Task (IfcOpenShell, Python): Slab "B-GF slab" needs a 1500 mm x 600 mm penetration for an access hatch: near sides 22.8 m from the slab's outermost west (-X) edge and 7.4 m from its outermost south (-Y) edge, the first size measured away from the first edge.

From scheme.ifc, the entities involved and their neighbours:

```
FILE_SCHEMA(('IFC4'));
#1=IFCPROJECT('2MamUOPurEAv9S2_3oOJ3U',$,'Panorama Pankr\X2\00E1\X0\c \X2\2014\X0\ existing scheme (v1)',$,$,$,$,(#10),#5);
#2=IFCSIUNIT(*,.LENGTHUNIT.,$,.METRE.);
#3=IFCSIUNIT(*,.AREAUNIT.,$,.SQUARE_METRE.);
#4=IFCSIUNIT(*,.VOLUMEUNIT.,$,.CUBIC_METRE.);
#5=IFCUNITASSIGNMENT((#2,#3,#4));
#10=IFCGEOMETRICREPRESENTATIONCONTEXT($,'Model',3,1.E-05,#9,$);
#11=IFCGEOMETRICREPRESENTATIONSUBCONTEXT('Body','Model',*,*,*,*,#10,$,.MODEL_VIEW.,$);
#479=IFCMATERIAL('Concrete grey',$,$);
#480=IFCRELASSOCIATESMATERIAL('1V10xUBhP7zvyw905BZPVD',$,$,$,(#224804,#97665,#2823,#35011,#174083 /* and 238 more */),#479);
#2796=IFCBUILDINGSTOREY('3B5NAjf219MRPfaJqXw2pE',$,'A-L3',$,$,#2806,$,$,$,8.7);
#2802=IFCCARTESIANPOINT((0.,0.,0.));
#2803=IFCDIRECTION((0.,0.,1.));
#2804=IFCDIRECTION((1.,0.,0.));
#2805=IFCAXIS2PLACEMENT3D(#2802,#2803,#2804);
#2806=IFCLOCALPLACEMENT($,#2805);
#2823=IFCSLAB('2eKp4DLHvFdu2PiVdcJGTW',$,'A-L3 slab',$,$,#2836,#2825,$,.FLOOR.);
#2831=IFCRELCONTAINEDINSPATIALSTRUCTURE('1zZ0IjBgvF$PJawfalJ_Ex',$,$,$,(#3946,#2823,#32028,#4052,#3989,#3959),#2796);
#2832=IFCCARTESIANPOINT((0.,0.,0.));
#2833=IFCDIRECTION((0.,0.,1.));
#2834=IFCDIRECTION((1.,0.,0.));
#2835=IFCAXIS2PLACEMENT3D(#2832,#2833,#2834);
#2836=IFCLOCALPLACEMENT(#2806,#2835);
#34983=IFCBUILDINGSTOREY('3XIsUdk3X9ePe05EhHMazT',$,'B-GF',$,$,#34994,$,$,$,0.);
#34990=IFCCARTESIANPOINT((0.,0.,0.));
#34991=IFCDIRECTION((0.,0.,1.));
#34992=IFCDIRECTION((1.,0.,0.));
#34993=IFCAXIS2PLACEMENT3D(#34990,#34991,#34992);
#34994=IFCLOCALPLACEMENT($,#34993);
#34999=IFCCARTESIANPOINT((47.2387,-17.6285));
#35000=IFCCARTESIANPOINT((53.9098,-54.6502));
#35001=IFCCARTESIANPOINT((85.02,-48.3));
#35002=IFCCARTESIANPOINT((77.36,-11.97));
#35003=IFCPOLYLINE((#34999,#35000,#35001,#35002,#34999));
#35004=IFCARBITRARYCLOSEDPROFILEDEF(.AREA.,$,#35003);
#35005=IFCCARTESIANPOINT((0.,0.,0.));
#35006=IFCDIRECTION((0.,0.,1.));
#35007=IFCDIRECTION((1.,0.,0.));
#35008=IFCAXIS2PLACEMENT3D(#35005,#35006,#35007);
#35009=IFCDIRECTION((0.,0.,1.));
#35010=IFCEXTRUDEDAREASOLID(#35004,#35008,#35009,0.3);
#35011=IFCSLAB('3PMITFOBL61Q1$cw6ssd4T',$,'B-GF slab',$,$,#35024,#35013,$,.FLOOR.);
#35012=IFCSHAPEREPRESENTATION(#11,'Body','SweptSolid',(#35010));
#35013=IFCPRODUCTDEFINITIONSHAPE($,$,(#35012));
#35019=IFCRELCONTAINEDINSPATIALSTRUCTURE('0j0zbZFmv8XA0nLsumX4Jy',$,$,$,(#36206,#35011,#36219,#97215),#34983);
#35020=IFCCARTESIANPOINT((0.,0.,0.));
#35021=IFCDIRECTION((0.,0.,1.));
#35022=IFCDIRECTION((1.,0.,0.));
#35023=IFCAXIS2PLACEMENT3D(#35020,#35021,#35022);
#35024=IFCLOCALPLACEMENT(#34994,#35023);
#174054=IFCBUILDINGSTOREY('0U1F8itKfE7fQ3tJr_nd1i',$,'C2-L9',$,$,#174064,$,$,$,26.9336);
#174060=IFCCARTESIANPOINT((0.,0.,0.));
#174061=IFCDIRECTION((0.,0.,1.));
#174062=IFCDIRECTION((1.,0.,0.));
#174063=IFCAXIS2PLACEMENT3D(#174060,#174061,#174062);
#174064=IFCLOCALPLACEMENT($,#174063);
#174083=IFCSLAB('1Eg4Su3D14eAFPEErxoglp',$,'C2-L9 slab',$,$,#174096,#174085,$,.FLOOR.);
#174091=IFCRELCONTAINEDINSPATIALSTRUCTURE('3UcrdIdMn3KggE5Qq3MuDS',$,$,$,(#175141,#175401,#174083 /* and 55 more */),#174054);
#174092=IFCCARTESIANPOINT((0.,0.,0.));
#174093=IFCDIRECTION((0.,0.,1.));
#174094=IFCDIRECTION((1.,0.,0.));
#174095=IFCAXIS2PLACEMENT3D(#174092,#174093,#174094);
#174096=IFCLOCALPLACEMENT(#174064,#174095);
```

```python
import numpy as np
import ifcopenshell
import ifcopenshell.api.feature
import ifcopenshell.api.geometry
import ifcopenshell.api.root
import ifcopenshell.geom
import ifcopenshell.util.placement
import ifcopenshell.util.representation
import ifcopenshell.util.shape
import ifcopenshell.util.unit

model = ifcopenshell.open("scheme.ifc")
unit_scale = ifcopenshell.util.unit.calculate_unit_scale(model)
settings = ifcopenshell.geom.settings()


def volume(element):
    """Net volume in cubic metres, openings subtracted."""
    shape = ifcopenshell.geom.create_shape(settings, element)
    return ifcopenshell.util.shape.get_volume(shape.geometry)


slab = model.by_guid("3PMITFOBL61Q1$cw6ssd4T")
before = volume(slab)

# Extent in the slab's own axes, in metres. The edges named are its -X and -Y sides.
slab_shape = ifcopenshell.geom.create_shape(settings, slab)
vertices = ifcopenshell.util.shape.get_vertices(slab_shape.geometry)
x_min, y_min, bottom = vertices.min(axis=0)
top = vertices[:, 2].max()

opening = ifcopenshell.api.root.create_entity(model, ifc_class="IfcOpeningElement", name="Access hatch opening", predefined_type="OPENING")
context = ifcopenshell.util.representation.get_context(model, "Model", "Body", "MODEL_VIEW")
width, depth = 1.5, 0.6
outline = [(0.0, 0.0), (width, 0.0), (width, depth), (0.0, depth), (0.0, 0.0)]
# Overshoot both faces by 50 mm so the cut is clean.
shape = ifcopenshell.api.geometry.add_slab_representation(
    model, context=context, depth=top - bottom + 0.1, polyline=outline
)
ifcopenshell.api.geometry.assign_representation(model, product=opening, representation=shape)

matrix = ifcopenshell.util.placement.get_local_placement(slab.ObjectPlacement)
matrix[:, 3] = matrix @ np.append(np.array([x_min + 22.8, y_min + 7.4, bottom - 0.05]) / unit_scale, 1.0)
ifcopenshell.api.geometry.edit_object_placement(model, product=opening, matrix=matrix, is_si=False)
ifcopenshell.api.feature.add_feature(model, feature=opening, element=slab)

after = volume(slab)

print(f"slab volume {before:.3f} -> {after:.3f} m3")

model.write("scheme-out.ifc")
```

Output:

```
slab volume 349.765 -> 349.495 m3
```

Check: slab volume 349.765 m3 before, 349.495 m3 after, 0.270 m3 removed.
